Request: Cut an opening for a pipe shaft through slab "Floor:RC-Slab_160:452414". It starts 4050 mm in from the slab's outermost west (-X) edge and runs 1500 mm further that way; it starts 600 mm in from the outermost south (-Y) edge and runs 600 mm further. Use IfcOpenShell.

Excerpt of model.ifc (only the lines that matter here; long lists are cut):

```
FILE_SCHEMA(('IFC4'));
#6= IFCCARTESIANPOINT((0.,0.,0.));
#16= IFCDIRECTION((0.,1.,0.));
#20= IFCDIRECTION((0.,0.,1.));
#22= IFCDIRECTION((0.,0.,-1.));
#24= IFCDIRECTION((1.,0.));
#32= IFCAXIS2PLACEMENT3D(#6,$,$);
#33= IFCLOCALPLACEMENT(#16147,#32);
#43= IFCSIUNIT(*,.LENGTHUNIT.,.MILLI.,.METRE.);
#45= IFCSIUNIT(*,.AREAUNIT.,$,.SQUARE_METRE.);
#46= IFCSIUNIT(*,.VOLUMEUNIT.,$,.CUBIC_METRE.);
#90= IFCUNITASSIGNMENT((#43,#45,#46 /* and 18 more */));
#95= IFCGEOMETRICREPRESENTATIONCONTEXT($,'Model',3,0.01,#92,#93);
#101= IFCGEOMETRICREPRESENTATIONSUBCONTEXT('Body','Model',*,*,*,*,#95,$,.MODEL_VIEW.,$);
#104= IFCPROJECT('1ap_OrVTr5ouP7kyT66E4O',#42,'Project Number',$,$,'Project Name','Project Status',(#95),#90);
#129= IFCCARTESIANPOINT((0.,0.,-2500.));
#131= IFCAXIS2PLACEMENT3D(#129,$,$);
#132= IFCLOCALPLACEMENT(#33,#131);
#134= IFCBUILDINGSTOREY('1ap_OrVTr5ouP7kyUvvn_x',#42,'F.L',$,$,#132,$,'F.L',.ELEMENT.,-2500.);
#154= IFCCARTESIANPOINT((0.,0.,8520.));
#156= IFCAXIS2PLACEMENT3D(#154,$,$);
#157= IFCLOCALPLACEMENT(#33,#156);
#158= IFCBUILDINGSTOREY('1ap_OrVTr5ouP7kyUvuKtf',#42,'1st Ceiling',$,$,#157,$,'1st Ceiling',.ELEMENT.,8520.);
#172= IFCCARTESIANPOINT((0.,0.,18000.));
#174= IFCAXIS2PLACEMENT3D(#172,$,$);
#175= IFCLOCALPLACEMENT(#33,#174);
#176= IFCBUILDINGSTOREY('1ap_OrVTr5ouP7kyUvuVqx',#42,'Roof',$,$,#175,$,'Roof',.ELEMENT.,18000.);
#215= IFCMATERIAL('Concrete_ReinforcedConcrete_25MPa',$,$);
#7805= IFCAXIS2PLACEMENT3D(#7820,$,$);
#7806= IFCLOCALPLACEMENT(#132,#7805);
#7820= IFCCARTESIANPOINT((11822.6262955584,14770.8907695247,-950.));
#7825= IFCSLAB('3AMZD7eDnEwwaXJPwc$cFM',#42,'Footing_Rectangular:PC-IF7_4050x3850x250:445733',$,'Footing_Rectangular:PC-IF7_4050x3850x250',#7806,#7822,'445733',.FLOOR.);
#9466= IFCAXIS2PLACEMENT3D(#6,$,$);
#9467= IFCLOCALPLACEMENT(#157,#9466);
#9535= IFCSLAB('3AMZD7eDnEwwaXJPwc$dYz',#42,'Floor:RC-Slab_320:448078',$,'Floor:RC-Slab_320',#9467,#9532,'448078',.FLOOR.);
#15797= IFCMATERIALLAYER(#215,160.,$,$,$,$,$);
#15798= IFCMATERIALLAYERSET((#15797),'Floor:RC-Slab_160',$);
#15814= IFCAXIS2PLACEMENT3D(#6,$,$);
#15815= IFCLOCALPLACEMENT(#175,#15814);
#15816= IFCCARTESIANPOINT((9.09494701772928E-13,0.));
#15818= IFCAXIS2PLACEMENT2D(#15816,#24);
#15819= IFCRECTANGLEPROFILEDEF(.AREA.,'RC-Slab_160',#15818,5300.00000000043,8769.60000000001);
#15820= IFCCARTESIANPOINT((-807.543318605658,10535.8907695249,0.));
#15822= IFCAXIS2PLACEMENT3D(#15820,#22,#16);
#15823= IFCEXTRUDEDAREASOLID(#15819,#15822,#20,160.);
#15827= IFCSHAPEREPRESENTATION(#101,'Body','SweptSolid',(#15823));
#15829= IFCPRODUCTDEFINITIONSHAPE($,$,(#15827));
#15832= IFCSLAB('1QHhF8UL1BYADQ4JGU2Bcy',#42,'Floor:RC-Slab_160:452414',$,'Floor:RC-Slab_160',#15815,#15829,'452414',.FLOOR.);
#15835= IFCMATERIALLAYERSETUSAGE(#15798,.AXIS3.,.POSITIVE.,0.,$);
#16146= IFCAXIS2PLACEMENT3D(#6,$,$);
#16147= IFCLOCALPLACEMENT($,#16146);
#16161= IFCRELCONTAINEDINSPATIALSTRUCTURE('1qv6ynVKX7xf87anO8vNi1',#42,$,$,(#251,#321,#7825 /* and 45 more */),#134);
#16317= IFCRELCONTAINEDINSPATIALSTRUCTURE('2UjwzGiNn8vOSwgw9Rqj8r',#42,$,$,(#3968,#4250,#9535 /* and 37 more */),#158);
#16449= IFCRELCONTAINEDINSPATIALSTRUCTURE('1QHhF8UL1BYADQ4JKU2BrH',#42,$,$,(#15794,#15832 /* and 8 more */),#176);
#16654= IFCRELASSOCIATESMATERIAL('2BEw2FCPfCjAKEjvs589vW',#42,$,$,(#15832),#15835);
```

```python
import numpy as np
import ifcopenshell
import ifcopenshell.api.feature
import ifcopenshell.api.geometry
import ifcopenshell.api.root
import ifcopenshell.geom
import ifcopenshell.util.placement
import ifcopenshell.util.representation
import ifcopenshell.util.shape
import ifcopenshell.util.unit

model = ifcopenshell.open("model.ifc")
unit_scale = ifcopenshell.util.unit.calculate_unit_scale(model)
settings = ifcopenshell.geom.settings()


def volume(element):
    """Net volume in cubic metres, openings subtracted."""
    shape = ifcopenshell.geom.create_shape(settings, element)
    return ifcopenshell.util.shape.get_volume(shape.geometry)


slab = model.by_guid("1QHhF8UL1BYADQ4JGU2Bcy")
before = volume(slab)

# Extent in the slab's own axes, in metres. The edges named are its -X and -Y sides.
slab_shape = ifcopenshell.geom.create_shape(settings, slab)
vertices = ifcopenshell.util.shape.get_vertices(slab_shape.geometry)
x_min, y_min, bottom = vertices.min(axis=0)
top = vertices[:, 2].max()

opening = ifcopenshell.api.root.create_entity(model, ifc_class="IfcOpeningElement", name="Pipe shaft opening", predefined_type="OPENING")
context = ifcopenshell.util.representation.get_context(model, "Model", "Body", "MODEL_VIEW")
width, depth = 1.5, 0.6
outline = [(0.0, 0.0), (width, 0.0), (width, depth), (0.0, depth), (0.0, 0.0)]
# Overshoot both faces by 50 mm so the cut is clean.
shape = ifcopenshell.api.geometry.add_slab_representation(
    model, context=context, depth=top - bottom + 0.1, polyline=outline
)
ifcopenshell.api.geometry.assign_representation(model, product=opening, representation=shape)

matrix = ifcopenshell.util.placement.get_local_placement(slab.ObjectPlacement)
matrix[:, 3] = matrix @ np.append(np.array([x_min + 4.05, y_min + 0.6, bottom - 0.05]) / unit_scale, 1.0)
ifcopenshell.api.geometry.edit_object_placement(model, product=opening, matrix=matrix, is_si=False)
ifcopenshell.api.feature.add_feature(model, feature=opening, element=slab)

after = volume(slab)

print(f"slab volume {before:.3f} -> {after:.3f} m3")

model.write("model_v2.ifc")
```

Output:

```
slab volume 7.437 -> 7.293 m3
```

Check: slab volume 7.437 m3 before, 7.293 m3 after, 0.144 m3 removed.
